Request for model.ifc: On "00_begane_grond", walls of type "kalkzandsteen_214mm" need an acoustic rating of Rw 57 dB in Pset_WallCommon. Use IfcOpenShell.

First a look at what the model holds.

```python
import ifcopenshell
import ifcopenshell.util.element

model = ifcopenshell.open("model.ifc")
print(model.schema)
storey = next(s for s in model.by_type("IfcBuildingStorey") if s.Name == "00_begane_grond")
walls = [e for e in ifcopenshell.util.element.get_decomposition(storey) if e.is_a("IfcWall")]
seen = {}
for e in walls:
    element_type = ifcopenshell.util.element.get_type(e)
    key = (element_type.Name if element_type != e and element_type else None, ifcopenshell.util.element.get_pset(e, "Pset_WallCommon", "AcousticRating"))
    seen[key] = seen.get(key, 0) + 1
for (name, value), count in sorted(seen.items(), key=str):
    print(count, "x", name, "|", value)
```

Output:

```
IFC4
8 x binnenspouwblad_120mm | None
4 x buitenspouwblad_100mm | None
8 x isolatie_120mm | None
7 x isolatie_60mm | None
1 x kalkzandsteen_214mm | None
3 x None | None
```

```python
import ifcopenshell
import ifcopenshell.api.pset
import ifcopenshell.util.element

model = ifcopenshell.open("model.ifc")

storey = next(s for s in model.by_type("IfcBuildingStorey") if s.Name == "00_begane_grond")
walls = [e for e in ifcopenshell.util.element.get_decomposition(storey) if e.is_a("IfcWall")]

count = 0
for e in walls:
    element_type = ifcopenshell.util.element.get_type(e)
    if element_type in (None, e) or element_type.Name != "kalkzandsteen_214mm":
        continue
    # add_pset returns the element's existing set when there is one.
    pset = ifcopenshell.api.pset.add_pset(model, product=e, name="Pset_WallCommon")
    ifcopenshell.api.pset.edit_pset(model, pset=pset, properties={"AcousticRating": "Rw 57 dB"})
    count += 1

print(count, "walls updated")

model.write("model_edited.ifc")
```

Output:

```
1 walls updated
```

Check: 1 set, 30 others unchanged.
